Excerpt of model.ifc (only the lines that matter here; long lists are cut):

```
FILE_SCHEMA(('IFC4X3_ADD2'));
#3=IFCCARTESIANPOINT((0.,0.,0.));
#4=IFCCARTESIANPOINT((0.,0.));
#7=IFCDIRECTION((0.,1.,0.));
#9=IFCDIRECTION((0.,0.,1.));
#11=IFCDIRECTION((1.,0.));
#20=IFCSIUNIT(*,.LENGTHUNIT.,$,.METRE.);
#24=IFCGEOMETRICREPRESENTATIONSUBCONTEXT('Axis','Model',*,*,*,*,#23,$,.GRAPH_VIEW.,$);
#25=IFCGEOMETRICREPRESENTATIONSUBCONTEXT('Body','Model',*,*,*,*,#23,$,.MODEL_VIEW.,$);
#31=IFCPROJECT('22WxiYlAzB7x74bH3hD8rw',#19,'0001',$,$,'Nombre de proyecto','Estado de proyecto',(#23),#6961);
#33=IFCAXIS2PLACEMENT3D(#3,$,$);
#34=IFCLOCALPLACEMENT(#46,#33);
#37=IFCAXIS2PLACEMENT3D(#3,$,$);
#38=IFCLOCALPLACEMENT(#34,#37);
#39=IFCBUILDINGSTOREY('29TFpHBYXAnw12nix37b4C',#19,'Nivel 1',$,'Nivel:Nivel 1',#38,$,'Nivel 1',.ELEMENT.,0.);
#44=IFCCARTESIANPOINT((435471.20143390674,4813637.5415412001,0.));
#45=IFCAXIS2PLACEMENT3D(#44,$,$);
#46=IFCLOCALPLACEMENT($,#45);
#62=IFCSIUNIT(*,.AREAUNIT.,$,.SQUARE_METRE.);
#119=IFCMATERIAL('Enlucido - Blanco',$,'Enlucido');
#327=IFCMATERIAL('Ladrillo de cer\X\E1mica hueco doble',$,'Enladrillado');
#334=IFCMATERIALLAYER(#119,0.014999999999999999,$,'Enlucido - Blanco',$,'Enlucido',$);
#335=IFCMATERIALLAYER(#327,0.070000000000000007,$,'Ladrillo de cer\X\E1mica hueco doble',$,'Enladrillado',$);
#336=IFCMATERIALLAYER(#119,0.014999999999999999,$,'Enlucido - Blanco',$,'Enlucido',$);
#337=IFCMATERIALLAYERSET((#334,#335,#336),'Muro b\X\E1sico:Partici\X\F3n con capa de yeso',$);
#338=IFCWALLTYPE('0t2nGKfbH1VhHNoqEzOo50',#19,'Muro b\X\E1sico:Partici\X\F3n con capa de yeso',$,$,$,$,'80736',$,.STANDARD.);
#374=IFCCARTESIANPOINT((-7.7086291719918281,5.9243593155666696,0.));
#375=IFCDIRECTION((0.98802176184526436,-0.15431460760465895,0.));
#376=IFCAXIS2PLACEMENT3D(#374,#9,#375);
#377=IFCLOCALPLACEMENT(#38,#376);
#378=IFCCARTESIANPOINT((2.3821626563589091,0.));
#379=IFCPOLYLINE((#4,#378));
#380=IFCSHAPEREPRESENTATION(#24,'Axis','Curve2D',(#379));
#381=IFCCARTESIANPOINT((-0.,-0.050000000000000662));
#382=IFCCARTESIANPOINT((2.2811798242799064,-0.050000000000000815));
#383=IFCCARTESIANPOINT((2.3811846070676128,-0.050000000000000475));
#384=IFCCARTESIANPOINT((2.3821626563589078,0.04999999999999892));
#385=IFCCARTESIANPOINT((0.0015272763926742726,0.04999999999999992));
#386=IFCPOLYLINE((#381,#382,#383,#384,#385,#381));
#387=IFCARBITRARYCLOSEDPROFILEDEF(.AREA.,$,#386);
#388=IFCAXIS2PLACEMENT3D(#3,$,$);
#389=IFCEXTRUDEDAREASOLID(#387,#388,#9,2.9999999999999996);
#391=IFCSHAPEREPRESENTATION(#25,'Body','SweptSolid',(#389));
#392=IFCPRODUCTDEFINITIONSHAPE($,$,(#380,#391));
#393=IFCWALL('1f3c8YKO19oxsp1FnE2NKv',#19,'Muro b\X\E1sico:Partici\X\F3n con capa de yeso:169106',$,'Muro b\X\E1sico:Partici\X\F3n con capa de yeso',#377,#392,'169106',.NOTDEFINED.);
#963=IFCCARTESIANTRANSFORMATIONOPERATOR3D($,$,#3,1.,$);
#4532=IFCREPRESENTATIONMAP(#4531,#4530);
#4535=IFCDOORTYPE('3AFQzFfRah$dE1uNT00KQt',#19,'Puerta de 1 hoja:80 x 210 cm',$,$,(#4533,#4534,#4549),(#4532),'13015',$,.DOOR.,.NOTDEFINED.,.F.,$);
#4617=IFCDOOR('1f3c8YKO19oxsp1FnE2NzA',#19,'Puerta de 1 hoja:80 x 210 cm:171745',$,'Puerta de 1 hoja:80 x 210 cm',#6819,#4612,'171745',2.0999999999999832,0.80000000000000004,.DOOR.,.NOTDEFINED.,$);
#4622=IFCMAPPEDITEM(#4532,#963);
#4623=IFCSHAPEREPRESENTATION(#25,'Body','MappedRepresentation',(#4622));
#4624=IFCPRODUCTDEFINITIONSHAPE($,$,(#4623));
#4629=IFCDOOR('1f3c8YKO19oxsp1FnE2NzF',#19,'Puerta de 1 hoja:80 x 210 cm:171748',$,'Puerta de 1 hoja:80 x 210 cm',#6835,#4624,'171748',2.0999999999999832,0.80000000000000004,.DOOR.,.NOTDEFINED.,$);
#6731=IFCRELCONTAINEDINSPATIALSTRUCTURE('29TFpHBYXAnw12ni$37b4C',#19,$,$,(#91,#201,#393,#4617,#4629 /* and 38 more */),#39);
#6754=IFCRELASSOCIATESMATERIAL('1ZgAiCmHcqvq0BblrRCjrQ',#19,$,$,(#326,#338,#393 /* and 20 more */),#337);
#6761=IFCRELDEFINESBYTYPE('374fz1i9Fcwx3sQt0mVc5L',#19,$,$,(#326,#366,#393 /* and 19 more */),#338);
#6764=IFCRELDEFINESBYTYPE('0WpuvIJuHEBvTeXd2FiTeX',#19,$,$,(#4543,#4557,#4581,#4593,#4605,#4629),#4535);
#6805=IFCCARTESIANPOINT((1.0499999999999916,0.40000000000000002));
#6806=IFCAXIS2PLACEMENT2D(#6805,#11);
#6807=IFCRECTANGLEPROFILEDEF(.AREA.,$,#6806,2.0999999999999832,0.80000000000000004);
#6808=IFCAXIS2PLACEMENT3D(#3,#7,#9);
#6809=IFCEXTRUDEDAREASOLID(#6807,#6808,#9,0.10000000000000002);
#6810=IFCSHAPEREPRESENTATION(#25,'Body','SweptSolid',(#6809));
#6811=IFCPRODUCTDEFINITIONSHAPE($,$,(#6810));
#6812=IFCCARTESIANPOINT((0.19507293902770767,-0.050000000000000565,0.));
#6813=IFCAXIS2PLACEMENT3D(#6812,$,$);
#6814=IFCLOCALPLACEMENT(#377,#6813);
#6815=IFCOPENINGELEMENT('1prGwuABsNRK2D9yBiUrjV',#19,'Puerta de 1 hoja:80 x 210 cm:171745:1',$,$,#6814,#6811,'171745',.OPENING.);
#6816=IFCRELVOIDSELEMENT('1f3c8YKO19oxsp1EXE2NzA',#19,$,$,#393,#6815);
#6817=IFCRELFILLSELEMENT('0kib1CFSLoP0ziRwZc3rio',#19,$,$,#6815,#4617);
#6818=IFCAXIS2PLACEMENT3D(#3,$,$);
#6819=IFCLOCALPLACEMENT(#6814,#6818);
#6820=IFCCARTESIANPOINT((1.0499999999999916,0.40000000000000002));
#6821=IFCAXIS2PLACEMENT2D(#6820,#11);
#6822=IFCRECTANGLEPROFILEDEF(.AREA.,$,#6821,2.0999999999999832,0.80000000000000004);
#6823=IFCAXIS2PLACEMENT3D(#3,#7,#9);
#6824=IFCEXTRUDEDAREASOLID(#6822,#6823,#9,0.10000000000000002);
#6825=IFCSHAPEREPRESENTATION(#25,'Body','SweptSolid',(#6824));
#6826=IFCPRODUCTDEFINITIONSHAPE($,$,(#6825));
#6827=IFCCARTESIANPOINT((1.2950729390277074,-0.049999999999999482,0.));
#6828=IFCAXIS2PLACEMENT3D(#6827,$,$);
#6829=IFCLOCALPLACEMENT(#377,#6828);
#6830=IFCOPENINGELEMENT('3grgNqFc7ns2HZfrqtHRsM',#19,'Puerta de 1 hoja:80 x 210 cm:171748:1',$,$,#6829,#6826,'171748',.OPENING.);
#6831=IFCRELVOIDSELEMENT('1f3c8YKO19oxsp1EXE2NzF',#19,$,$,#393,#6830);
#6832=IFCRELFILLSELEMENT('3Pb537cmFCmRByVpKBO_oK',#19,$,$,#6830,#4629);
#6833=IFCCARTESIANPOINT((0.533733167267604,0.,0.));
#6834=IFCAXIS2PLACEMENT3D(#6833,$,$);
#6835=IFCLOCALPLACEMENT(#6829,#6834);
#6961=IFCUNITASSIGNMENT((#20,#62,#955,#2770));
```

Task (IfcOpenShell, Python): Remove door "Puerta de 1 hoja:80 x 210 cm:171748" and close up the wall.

```python
import ifcopenshell
import ifcopenshell.api.feature
import ifcopenshell.api.root
import ifcopenshell.geom
import ifcopenshell.util.shape

model = ifcopenshell.open("model.ifc")
settings = ifcopenshell.geom.settings()


def volume(element):
    """Net volume in cubic metres, openings subtracted."""
    shape = ifcopenshell.geom.create_shape(settings, element)
    return ifcopenshell.util.shape.get_volume(shape.geometry)


door = model.by_id(4629)
opening = door.FillsVoids[0].RelatingOpeningElement
wall = opening.VoidsElements[0].RelatingBuildingElement
before = volume(wall)

ifcopenshell.api.root.remove_product(model, product=door)
ifcopenshell.api.feature.remove_feature(model, feature=opening)

after = volume(wall)

print(f"wall volume {before:.3f} -> {after:.3f} m3")

model.write("model-out.ifc")
```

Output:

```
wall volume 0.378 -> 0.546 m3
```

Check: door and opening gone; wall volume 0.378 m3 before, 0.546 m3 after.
